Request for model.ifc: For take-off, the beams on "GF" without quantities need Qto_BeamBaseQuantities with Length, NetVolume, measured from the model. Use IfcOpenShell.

First a look at what the model holds.

```python
import ifcopenshell
import ifcopenshell.util.element
import ifcopenshell.util.unit

model = ifcopenshell.open("model.ifc")
print(model.schema)
for unit_type in ("LENGTHUNIT", "AREAUNIT", "VOLUMEUNIT"):
    print(unit_type, ifcopenshell.util.unit.calculate_unit_scale(model, unit_type))
storey = next(s for s in model.by_type("IfcBuildingStorey") if s.Name == "GF")
beams = [e for e in ifcopenshell.util.element.get_decomposition(storey) if e.is_a("IfcBeam")]
for e in sorted(beams, key=lambda e: e.id()):
    print(e.id(), e.is_a(), e.Name, list(ifcopenshell.util.element.get_psets(e, qtos_only=True)), sep=" | ")
```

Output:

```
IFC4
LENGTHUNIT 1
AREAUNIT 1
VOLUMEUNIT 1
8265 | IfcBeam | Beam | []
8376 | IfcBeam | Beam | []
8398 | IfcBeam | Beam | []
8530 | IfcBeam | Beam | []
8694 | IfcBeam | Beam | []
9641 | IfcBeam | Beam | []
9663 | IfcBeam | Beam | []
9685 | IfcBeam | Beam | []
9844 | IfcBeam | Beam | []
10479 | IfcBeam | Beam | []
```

```python
import ifcopenshell
import ifcopenshell.api.pset
import ifcopenshell.geom
import ifcopenshell.util.element
import ifcopenshell.util.shape
import ifcopenshell.util.unit

model = ifcopenshell.open("model.ifc")
unit_scale = ifcopenshell.util.unit.calculate_unit_scale(model)
volume_scale = ifcopenshell.util.unit.calculate_unit_scale(model, "VOLUMEUNIT")
settings = ifcopenshell.geom.settings()

storey = next(s for s in model.by_type("IfcBuildingStorey") if s.Name == "GF")
beams = [e for e in ifcopenshell.util.element.get_decomposition(storey) if e.is_a("IfcBeam")]

for e in sorted(beams, key=lambda e: e.id()):
    if ifcopenshell.util.element.get_psets(e, qtos_only=True, should_inherit=False):
        continue
    # Geometry comes back in metres, in the element's own axes.
    shape = ifcopenshell.geom.create_shape(settings, e)
    values = {
        "Length": ifcopenshell.util.shape.get_max_xyz(shape.geometry) / unit_scale,
        "NetVolume": ifcopenshell.util.shape.get_volume(shape.geometry) / volume_scale,
    }
    qto = ifcopenshell.api.pset.add_qto(model, product=e, name="Qto_BeamBaseQuantities")
    ifcopenshell.api.pset.edit_qto(model, qto=qto, properties=values)
    print(e.id(), {k: round(v, 3) for k, v in values.items()})

model.write("model_v2.ifc")
```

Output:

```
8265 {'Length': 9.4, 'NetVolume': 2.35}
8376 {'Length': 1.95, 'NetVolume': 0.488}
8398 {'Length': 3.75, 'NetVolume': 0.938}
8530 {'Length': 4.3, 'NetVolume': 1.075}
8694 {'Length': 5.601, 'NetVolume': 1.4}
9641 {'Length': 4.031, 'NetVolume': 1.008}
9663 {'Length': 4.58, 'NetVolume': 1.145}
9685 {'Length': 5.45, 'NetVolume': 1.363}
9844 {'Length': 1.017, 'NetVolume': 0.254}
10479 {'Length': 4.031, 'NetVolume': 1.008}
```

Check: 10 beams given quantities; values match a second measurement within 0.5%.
